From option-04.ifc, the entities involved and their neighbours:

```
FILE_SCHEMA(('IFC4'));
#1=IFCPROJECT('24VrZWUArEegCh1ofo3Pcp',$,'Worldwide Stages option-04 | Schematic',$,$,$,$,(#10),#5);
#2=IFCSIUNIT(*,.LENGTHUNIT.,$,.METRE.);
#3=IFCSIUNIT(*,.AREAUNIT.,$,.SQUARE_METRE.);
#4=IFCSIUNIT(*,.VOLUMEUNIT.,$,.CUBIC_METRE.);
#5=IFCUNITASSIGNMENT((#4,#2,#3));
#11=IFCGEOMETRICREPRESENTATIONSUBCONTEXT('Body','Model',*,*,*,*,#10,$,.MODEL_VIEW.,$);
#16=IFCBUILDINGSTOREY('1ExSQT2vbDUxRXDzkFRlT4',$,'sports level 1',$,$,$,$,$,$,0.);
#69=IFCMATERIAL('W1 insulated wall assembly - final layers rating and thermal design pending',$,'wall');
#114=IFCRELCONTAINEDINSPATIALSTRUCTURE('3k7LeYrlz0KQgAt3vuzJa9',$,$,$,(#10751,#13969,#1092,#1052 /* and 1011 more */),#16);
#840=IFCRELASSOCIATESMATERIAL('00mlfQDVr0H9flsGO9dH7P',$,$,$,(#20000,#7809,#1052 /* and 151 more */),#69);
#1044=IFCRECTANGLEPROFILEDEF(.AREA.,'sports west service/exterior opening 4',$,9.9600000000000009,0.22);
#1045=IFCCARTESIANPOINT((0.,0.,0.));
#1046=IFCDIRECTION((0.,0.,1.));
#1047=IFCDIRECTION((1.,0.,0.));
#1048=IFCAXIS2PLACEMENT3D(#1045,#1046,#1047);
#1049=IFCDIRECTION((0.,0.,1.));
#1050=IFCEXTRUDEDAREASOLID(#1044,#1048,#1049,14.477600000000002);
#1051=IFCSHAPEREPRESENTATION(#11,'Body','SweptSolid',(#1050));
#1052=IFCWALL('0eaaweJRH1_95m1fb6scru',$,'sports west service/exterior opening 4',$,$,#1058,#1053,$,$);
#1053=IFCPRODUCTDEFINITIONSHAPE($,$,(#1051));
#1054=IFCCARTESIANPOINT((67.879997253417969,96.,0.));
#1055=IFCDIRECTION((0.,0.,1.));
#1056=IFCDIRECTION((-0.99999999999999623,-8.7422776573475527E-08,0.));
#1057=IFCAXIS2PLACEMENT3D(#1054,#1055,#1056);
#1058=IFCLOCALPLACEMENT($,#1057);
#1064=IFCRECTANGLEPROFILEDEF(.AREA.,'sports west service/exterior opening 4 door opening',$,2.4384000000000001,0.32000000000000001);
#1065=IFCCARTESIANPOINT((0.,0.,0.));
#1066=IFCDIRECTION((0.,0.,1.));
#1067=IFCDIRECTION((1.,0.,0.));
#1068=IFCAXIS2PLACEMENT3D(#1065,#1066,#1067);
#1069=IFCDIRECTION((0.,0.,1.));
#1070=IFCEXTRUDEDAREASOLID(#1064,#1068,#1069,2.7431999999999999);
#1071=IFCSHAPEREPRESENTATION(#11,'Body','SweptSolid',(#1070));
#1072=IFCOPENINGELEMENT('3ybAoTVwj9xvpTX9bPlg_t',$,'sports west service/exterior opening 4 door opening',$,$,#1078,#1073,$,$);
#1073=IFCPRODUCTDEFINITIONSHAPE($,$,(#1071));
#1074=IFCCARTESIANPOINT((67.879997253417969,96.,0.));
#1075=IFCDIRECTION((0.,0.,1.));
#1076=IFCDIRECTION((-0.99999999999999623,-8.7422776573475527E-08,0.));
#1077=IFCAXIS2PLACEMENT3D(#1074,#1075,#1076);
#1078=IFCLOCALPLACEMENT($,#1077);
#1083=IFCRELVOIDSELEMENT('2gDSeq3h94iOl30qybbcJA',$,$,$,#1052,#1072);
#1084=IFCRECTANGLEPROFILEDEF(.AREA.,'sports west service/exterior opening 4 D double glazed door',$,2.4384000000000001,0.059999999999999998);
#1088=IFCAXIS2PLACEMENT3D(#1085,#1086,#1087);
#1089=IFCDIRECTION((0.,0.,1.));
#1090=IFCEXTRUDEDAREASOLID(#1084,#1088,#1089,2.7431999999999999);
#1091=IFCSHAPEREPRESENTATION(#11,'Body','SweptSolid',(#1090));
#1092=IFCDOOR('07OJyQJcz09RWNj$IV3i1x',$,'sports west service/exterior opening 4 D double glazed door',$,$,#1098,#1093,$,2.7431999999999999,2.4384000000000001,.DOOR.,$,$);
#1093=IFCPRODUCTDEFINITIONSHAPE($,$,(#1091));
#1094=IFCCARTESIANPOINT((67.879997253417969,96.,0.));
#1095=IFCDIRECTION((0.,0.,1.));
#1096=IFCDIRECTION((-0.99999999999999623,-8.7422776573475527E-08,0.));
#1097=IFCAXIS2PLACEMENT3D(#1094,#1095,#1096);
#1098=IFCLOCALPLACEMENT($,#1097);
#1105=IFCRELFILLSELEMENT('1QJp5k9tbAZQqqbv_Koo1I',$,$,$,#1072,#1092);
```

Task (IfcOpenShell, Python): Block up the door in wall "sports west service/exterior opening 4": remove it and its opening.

```python
import ifcopenshell
import ifcopenshell.api.feature
import ifcopenshell.api.root
import ifcopenshell.geom
import ifcopenshell.util.shape

model = ifcopenshell.open("option-04.ifc")
settings = ifcopenshell.geom.settings()


def volume(element):
    """Net volume in cubic metres, openings subtracted."""
    shape = ifcopenshell.geom.create_shape(settings, element)
    return ifcopenshell.util.shape.get_volume(shape.geometry)


door = model.by_guid("07OJyQJcz09RWNj$IV3i1x")
opening = door.FillsVoids[0].RelatingOpeningElement
wall = opening.VoidsElements[0].RelatingBuildingElement
before = volume(wall)

ifcopenshell.api.root.remove_product(model, product=door)
ifcopenshell.api.feature.remove_feature(model, feature=opening)

after = volume(wall)

print(f"wall volume {before:.3f} -> {after:.3f} m3")

model.write("option-04-out.ifc")
```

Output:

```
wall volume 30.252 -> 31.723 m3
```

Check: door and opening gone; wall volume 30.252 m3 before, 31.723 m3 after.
